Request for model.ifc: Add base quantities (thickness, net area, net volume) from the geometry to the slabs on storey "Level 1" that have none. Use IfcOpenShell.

First a look at what the model holds.

```python
import ifcopenshell
import ifcopenshell.util.element
import ifcopenshell.util.unit

model = ifcopenshell.open("model.ifc")
print(model.schema)
for unit_type in ("LENGTHUNIT", "AREAUNIT", "VOLUMEUNIT"):
    print(unit_type, ifcopenshell.util.unit.calculate_unit_scale(model, unit_type))
storey = next(s for s in model.by_type("IfcBuildingStorey") if s.Name == "Level 1")
slabs = [e for e in ifcopenshell.util.element.get_decomposition(storey) if e.is_a("IfcSlab")]
for e in sorted(slabs, key=lambda e: e.id()):
    print(e.id(), e.is_a(), e.Name, list(ifcopenshell.util.element.get_psets(e, qtos_only=True)), sep=" | ")
```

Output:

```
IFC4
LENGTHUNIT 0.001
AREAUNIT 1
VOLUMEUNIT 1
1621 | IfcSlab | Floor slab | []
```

```python
import ifcopenshell
import ifcopenshell.api.pset
import ifcopenshell.geom
import ifcopenshell.util.element
import ifcopenshell.util.shape
import ifcopenshell.util.unit

model = ifcopenshell.open("model.ifc")
unit_scale = ifcopenshell.util.unit.calculate_unit_scale(model)
area_scale = ifcopenshell.util.unit.calculate_unit_scale(model, "AREAUNIT")
volume_scale = ifcopenshell.util.unit.calculate_unit_scale(model, "VOLUMEUNIT")
settings = ifcopenshell.geom.settings()

storey = next(s for s in model.by_type("IfcBuildingStorey") if s.Name == "Level 1")
slabs = [e for e in ifcopenshell.util.element.get_decomposition(storey) if e.is_a("IfcSlab")]

for e in sorted(slabs, key=lambda e: e.id()):
    if ifcopenshell.util.element.get_psets(e, qtos_only=True, should_inherit=False):
        continue
    # Geometry comes back in metres, in the element's own axes.
    shape = ifcopenshell.geom.create_shape(settings, e)
    values = {
        "Width": ifcopenshell.util.shape.get_z(shape.geometry) / unit_scale,
        "NetArea": ifcopenshell.util.shape.get_footprint_area(shape.geometry) / area_scale,
        "NetVolume": ifcopenshell.util.shape.get_volume(shape.geometry) / volume_scale,
    }
    qto = ifcopenshell.api.pset.add_qto(model, product=e, name="Qto_SlabBaseQuantities")
    ifcopenshell.api.pset.edit_qto(model, qto=qto, properties=values)
    print(e.id(), {k: round(v, 3) for k, v in values.items()})

model.write("model_edited.ifc")
```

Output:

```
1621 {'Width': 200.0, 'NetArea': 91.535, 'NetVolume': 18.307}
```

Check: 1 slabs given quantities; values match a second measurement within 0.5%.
